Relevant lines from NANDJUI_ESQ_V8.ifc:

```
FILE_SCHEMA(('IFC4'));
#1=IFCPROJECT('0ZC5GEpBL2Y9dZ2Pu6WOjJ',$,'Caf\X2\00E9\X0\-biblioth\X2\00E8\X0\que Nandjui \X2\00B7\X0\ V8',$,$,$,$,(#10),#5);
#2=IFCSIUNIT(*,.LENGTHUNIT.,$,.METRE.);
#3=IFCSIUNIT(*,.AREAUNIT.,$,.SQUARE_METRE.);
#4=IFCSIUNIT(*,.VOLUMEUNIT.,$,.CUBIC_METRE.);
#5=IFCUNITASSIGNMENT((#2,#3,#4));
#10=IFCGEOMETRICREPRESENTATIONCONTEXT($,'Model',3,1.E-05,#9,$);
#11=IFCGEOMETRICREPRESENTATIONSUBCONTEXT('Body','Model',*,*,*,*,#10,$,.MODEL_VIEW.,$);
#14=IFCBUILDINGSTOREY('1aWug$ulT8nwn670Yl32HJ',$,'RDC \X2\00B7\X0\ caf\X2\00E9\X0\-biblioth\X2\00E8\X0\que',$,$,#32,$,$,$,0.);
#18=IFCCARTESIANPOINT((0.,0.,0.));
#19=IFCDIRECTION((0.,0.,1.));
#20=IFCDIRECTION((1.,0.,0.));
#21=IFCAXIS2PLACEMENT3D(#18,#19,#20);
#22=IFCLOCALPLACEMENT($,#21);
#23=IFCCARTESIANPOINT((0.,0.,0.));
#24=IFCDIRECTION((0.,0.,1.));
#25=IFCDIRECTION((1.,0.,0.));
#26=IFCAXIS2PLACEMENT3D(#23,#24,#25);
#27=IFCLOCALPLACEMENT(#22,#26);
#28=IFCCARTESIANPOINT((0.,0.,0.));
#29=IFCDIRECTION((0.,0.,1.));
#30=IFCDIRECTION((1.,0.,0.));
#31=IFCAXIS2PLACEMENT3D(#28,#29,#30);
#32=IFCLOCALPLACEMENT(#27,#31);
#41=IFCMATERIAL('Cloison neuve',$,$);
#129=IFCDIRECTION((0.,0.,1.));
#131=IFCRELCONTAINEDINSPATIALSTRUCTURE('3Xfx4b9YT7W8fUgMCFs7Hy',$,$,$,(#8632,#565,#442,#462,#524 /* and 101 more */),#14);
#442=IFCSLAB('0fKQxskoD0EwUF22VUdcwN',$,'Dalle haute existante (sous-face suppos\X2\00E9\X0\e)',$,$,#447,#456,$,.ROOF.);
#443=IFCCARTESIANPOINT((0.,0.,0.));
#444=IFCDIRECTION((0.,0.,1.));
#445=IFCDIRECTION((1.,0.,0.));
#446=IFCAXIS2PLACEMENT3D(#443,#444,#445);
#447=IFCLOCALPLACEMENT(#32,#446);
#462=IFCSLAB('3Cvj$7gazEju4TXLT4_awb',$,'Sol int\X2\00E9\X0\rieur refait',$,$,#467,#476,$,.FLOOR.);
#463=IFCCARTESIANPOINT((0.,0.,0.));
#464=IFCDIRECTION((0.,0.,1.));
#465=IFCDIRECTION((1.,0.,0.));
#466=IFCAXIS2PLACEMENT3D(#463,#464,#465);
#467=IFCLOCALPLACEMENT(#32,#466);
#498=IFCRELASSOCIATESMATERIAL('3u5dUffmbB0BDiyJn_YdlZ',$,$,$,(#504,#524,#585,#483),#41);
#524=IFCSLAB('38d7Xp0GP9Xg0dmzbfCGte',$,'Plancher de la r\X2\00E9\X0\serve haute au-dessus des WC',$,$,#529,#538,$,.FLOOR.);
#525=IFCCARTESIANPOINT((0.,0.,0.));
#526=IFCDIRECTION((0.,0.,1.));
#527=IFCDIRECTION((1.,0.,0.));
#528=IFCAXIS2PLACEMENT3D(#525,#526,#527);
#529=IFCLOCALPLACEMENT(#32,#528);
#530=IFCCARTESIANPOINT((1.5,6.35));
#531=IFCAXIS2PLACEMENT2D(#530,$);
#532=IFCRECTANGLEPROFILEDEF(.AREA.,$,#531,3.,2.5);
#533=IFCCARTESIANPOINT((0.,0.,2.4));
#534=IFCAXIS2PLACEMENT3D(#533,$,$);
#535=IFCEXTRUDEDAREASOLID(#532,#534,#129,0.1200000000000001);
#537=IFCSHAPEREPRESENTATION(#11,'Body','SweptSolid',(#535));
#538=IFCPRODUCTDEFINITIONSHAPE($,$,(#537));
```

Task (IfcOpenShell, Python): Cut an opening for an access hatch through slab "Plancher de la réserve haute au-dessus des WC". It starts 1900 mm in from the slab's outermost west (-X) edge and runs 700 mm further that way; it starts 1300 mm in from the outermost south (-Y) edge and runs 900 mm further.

```python
import numpy as np
import ifcopenshell
import ifcopenshell.api.feature
import ifcopenshell.api.geometry
import ifcopenshell.api.root
import ifcopenshell.geom
import ifcopenshell.util.placement
import ifcopenshell.util.representation
import ifcopenshell.util.shape
import ifcopenshell.util.unit

model = ifcopenshell.open("NANDJUI_ESQ_V8.ifc")
unit_scale = ifcopenshell.util.unit.calculate_unit_scale(model)
settings = ifcopenshell.geom.settings()


def volume(element):
    """Net volume in cubic metres, openings subtracted."""
    shape = ifcopenshell.geom.create_shape(settings, element)
    return ifcopenshell.util.shape.get_volume(shape.geometry)


slab = model.by_guid("38d7Xp0GP9Xg0dmzbfCGte")
before = volume(slab)

# Extent in the slab's own axes, in metres. The edges named are its -X and -Y sides.
slab_shape = ifcopenshell.geom.create_shape(settings, slab)
vertices = ifcopenshell.util.shape.get_vertices(slab_shape.geometry)
x_min, y_min, bottom = vertices.min(axis=0)
top = vertices[:, 2].max()

opening = ifcopenshell.api.root.create_entity(model, ifc_class="IfcOpeningElement", name="Access hatch opening", predefined_type="OPENING")
context = ifcopenshell.util.representation.get_context(model, "Model", "Body", "MODEL_VIEW")
width, depth = 0.7, 0.9
outline = [(0.0, 0.0), (width, 0.0), (width, depth), (0.0, depth), (0.0, 0.0)]
# Overshoot both faces by 50 mm so the cut is clean.
shape = ifcopenshell.api.geometry.add_slab_representation(
    model, context=context, depth=top - bottom + 0.1, polyline=outline
)
ifcopenshell.api.geometry.assign_representation(model, product=opening, representation=shape)

matrix = ifcopenshell.util.placement.get_local_placement(slab.ObjectPlacement)
matrix[:, 3] = matrix @ np.append(np.array([x_min + 1.9, y_min + 1.3, bottom - 0.05]) / unit_scale, 1.0)
ifcopenshell.api.geometry.edit_object_placement(model, product=opening, matrix=matrix, is_si=False)
ifcopenshell.api.feature.add_feature(model, feature=opening, element=slab)

after = volume(slab)

print(f"slab volume {before:.3f} -> {after:.3f} m3")

model.write("NANDJUI_ESQ_V8_rev.ifc")
```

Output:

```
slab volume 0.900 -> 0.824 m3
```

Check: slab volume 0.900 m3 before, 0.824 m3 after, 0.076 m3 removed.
